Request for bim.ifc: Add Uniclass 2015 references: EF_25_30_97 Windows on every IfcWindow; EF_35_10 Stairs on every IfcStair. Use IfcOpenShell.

First a look at what the model holds.

```python
import ifcopenshell

model = ifcopenshell.open("bim.ifc")
print(model.schema)
print("classifications:", [c.Name for c in model.by_type("IfcClassification")])
for ifc_class in ("IfcDoor", "IfcRoof", "IfcStair", "IfcWall", "IfcWindow"):
    print(ifc_class, len(model.by_type(ifc_class)))
```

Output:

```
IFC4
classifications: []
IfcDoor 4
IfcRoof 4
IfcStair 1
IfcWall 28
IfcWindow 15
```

```python
import ifcopenshell
import ifcopenshell.api.classification

model = ifcopenshell.open("bim.ifc")

system = ifcopenshell.api.classification.add_classification(model, classification="Uniclass 2015")

codes = {
    "IfcWindow": ("EF_25_30_97", "Windows"),
    "IfcStair": ("EF_35_10", "Stairs"),
}
for ifc_class, (code, name) in codes.items():
    products = model.by_type(ifc_class)
    ifcopenshell.api.classification.add_reference(
        model, products=products, classification=system, identification=code, name=name
    )
    print(code, len(products))

model.write("bim-out.ifc")
```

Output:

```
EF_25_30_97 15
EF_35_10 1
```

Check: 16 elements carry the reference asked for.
